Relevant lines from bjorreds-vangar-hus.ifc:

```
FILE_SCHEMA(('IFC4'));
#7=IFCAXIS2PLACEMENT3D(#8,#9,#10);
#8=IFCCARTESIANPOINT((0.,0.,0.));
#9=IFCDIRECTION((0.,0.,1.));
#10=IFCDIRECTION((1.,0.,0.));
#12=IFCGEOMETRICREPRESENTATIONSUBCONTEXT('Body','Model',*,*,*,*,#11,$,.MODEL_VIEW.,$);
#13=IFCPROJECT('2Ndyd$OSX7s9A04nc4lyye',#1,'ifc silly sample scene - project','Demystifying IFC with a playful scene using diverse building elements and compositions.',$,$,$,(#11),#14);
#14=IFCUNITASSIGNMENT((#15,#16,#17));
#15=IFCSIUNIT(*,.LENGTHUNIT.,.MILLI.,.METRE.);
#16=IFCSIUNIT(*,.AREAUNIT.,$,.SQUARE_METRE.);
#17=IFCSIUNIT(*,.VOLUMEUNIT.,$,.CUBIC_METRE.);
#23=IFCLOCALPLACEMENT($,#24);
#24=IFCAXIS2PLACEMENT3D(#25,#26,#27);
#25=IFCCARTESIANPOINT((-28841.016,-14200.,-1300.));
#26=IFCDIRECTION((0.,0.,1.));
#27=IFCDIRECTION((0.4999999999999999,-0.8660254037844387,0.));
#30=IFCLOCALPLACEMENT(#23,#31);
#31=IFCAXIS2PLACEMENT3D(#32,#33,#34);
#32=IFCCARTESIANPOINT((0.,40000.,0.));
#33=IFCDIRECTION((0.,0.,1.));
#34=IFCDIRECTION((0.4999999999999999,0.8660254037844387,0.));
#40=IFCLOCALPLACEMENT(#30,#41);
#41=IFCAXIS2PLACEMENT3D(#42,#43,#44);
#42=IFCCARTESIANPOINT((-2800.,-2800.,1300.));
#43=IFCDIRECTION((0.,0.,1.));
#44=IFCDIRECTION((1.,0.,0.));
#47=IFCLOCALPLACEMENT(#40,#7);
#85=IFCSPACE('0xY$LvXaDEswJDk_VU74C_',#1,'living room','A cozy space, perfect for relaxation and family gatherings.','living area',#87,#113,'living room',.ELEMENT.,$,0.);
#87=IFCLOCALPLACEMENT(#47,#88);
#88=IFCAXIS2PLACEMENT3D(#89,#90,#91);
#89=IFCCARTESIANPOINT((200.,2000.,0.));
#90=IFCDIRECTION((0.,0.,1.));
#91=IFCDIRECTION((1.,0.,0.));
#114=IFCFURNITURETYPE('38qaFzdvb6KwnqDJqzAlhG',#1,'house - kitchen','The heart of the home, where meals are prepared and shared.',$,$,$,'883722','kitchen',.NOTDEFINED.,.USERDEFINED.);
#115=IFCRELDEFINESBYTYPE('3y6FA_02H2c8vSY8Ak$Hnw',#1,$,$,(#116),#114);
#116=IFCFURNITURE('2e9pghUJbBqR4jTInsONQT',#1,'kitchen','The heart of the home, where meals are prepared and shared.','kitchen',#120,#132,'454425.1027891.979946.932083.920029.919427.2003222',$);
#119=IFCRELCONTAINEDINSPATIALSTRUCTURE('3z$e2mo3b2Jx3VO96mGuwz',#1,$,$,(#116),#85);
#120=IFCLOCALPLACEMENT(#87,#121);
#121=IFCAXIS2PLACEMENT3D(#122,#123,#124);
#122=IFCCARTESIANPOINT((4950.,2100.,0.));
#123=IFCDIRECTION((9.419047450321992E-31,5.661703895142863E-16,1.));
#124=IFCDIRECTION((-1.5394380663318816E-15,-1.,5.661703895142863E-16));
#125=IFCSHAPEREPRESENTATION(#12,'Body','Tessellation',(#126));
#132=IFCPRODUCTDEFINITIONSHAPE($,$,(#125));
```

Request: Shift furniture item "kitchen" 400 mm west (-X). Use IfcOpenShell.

```python
import ifcopenshell
import ifcopenshell.api.geometry
import ifcopenshell.util.placement
import ifcopenshell.util.unit

model = ifcopenshell.open("bjorreds-vangar-hus.ifc")
unit_scale = ifcopenshell.util.unit.calculate_unit_scale(model)

item = model.by_id(116)
matrix = ifcopenshell.util.placement.get_local_placement(item.ObjectPlacement)
matrix[0, 3] -= 0.4 / unit_scale
ifcopenshell.api.geometry.edit_object_placement(model, product=item, matrix=matrix, is_si=False)

print(ifcopenshell.util.placement.get_local_placement(item.ObjectPlacement).round(3) + 0.0)

model.write("bjorreds-vangar-hus_edited.ifc")
```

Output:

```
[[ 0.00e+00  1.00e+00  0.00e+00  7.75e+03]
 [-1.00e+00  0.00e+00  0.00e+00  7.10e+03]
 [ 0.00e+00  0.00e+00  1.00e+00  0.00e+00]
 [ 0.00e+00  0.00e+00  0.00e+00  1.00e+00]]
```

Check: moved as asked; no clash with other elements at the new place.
